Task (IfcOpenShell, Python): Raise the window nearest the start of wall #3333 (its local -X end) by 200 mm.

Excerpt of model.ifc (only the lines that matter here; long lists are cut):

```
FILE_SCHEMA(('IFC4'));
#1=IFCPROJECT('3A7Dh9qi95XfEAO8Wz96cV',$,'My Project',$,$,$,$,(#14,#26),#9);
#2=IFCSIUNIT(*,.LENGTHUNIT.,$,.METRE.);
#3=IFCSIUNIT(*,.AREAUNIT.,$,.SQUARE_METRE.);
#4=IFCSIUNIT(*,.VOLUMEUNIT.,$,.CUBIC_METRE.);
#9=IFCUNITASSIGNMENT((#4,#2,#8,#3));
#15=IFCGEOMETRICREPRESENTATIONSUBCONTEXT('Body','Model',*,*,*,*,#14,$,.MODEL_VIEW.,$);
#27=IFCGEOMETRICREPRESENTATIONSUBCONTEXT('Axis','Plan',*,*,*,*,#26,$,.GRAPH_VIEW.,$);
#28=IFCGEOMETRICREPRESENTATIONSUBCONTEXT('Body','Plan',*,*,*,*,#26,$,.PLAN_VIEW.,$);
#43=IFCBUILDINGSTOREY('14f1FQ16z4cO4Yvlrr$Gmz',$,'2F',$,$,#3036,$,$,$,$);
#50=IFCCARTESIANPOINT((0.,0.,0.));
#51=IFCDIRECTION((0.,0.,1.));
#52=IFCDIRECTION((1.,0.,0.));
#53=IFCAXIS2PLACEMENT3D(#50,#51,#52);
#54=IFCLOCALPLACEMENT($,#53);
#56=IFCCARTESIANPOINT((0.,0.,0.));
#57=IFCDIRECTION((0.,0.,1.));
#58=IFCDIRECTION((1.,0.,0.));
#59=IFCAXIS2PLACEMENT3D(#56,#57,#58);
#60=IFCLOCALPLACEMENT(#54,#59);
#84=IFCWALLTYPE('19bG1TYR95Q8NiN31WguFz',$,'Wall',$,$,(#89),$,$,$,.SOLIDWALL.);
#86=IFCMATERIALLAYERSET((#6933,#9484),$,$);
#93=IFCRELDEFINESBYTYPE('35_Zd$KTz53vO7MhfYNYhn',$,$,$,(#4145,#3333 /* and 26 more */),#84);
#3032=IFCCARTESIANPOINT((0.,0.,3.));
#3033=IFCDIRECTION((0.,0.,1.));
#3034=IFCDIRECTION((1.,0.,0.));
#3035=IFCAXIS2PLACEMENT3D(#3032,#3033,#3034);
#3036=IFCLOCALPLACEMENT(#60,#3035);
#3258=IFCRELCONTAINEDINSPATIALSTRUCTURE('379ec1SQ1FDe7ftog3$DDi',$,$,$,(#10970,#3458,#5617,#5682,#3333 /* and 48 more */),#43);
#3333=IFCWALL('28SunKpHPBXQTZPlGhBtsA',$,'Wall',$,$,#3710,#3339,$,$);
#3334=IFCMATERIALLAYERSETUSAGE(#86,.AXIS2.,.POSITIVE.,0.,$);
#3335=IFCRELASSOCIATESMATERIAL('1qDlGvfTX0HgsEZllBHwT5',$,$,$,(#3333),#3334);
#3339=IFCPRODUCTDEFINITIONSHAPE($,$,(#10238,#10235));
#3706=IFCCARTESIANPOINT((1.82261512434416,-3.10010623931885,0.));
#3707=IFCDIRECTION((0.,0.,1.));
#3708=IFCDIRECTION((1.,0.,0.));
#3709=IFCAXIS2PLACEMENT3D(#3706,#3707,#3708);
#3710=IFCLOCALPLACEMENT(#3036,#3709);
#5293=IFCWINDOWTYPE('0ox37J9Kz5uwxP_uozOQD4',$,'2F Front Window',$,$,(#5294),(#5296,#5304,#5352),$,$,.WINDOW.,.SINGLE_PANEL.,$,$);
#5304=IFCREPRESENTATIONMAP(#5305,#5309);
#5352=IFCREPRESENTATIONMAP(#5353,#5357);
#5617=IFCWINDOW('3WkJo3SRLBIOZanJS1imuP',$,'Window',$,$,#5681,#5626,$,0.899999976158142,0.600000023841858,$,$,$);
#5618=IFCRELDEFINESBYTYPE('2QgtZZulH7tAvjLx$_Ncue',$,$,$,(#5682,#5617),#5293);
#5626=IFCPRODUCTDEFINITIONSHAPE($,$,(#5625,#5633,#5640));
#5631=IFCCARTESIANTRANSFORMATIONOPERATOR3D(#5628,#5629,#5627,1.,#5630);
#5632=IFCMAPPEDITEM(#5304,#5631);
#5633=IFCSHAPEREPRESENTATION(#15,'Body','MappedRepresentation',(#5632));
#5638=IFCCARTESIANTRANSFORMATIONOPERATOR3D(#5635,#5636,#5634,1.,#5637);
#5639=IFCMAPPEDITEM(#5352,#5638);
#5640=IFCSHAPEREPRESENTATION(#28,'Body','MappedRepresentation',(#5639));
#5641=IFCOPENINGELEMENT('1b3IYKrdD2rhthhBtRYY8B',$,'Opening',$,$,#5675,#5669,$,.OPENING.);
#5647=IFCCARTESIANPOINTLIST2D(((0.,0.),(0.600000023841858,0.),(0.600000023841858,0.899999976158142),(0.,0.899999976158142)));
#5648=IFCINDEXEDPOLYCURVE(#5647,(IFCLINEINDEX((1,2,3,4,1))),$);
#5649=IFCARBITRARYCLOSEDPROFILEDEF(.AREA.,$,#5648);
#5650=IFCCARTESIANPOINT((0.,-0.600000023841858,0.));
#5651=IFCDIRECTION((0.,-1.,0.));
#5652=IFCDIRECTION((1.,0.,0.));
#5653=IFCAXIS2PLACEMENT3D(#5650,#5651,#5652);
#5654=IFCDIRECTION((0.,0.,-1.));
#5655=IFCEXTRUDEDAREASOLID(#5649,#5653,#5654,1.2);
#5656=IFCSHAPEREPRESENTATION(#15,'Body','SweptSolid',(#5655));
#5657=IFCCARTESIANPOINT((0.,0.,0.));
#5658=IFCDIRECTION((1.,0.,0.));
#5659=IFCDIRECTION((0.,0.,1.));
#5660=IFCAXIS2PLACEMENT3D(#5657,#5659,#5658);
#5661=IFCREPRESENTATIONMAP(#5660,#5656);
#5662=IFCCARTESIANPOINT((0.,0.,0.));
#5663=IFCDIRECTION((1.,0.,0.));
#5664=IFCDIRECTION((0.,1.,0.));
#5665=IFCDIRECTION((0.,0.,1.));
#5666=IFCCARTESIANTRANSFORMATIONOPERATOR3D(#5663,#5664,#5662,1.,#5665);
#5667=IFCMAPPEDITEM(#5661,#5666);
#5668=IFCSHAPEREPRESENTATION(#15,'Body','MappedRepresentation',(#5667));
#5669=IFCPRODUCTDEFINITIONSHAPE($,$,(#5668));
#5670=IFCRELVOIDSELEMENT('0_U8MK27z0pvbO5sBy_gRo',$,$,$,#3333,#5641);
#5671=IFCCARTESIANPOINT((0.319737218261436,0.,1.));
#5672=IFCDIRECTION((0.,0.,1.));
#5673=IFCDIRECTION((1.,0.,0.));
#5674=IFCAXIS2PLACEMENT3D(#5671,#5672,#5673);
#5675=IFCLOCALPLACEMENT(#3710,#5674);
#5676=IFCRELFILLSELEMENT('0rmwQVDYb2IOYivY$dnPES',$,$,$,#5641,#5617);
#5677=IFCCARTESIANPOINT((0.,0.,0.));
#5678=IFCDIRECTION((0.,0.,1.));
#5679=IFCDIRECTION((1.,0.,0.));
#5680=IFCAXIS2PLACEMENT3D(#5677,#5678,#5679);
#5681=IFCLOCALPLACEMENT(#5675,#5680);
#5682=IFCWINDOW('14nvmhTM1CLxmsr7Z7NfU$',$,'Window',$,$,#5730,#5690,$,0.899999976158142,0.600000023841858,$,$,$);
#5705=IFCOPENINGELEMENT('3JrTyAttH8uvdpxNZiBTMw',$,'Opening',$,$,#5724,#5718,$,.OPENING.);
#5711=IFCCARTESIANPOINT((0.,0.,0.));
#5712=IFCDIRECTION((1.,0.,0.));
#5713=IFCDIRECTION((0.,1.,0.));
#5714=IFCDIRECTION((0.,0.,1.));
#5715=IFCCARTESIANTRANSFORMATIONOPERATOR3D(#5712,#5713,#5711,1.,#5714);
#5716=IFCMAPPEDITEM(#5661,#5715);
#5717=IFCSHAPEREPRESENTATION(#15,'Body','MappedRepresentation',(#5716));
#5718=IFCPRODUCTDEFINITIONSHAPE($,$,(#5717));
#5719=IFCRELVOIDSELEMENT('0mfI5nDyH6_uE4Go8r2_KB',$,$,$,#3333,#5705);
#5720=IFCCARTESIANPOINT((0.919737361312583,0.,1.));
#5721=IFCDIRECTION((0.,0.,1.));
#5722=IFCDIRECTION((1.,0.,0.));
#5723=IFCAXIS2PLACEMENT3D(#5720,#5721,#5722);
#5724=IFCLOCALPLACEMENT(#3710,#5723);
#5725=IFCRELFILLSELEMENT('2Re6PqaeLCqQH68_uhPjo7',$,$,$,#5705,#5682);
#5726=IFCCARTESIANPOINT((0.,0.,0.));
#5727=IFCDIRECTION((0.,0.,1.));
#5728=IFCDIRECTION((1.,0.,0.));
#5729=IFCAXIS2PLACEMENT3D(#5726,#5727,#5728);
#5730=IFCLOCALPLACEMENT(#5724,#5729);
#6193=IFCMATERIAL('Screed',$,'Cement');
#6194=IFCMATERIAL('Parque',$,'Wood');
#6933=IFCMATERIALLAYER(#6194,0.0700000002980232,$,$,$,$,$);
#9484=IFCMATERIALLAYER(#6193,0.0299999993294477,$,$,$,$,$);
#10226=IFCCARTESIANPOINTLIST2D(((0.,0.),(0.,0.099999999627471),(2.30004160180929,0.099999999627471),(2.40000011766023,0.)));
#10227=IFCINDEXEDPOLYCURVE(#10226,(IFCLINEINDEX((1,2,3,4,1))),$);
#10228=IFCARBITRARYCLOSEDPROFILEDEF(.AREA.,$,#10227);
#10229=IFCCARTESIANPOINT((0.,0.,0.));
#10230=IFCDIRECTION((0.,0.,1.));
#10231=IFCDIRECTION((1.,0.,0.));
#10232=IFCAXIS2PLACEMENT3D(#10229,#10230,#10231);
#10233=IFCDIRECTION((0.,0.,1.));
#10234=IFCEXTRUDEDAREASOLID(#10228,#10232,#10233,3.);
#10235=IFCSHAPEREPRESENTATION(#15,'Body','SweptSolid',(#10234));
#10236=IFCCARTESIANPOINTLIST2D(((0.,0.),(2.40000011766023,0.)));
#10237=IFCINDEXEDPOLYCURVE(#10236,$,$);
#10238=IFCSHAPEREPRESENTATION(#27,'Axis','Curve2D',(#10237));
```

```python
import numpy as np
import ifcopenshell
import ifcopenshell.api.geometry
import ifcopenshell.util.placement
import ifcopenshell.util.unit

model = ifcopenshell.open("model.ifc")
unit_scale = ifcopenshell.util.unit.calculate_unit_scale(model)

window = model.by_guid("3WkJo3SRLBIOZanJS1imuP")
opening = window.FillsVoids[0].RelatingOpeningElement
dz = 0.2 / unit_scale

shift = np.array([0.0, 0.0, dz])
# The window is placed relative to its opening, so it follows when the opening moves.
matrix = ifcopenshell.util.placement.get_local_placement(opening.ObjectPlacement)
matrix[:3, 3] += shift
ifcopenshell.api.geometry.edit_object_placement(
    model, product=opening, matrix=matrix, is_si=False, should_transform_children=True
)

print(f"moved by {dz * unit_scale:+.3f} m")

model.write("model-out.ifc")
```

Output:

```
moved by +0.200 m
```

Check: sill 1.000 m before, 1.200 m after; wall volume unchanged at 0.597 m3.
